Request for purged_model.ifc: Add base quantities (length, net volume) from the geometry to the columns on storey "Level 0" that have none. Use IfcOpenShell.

First a look at what the model holds.

```python
import ifcopenshell
import ifcopenshell.util.element
import ifcopenshell.util.unit

model = ifcopenshell.open("purged_model.ifc")
print(model.schema)
for unit_type in ("LENGTHUNIT", "AREAUNIT", "VOLUMEUNIT"):
    print(unit_type, ifcopenshell.util.unit.calculate_unit_scale(model, unit_type))
storey = next(s for s in model.by_type("IfcBuildingStorey") if s.Name == "Level 0")
columns = [e for e in ifcopenshell.util.element.get_decomposition(storey) if e.is_a("IfcColumn")]
for e in sorted(columns, key=lambda e: e.id()):
    print(e.id(), e.is_a(), e.Name, list(ifcopenshell.util.element.get_psets(e, qtos_only=True)), sep=" | ")
```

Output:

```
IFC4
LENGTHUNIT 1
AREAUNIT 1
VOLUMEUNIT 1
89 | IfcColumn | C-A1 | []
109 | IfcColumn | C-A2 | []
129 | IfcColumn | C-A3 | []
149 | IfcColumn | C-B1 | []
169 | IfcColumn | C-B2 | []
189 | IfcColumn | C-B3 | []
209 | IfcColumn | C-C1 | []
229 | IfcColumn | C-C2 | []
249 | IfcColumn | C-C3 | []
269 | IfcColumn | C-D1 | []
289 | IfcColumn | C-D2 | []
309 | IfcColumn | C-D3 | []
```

```python
import ifcopenshell
import ifcopenshell.api.pset
import ifcopenshell.geom
import ifcopenshell.util.element
import ifcopenshell.util.shape
import ifcopenshell.util.unit

model = ifcopenshell.open("purged_model.ifc")
unit_scale = ifcopenshell.util.unit.calculate_unit_scale(model)
volume_scale = ifcopenshell.util.unit.calculate_unit_scale(model, "VOLUMEUNIT")
settings = ifcopenshell.geom.settings()

storey = next(s for s in model.by_type("IfcBuildingStorey") if s.Name == "Level 0")
columns = [e for e in ifcopenshell.util.element.get_decomposition(storey) if e.is_a("IfcColumn")]

for e in sorted(columns, key=lambda e: e.id()):
    if ifcopenshell.util.element.get_psets(e, qtos_only=True, should_inherit=False):
        continue
    # Geometry comes back in metres, in the element's own axes.
    shape = ifcopenshell.geom.create_shape(settings, e)
    values = {
        "Length": ifcopenshell.util.shape.get_z(shape.geometry) / unit_scale,
        "NetVolume": ifcopenshell.util.shape.get_volume(shape.geometry) / volume_scale,
    }
    qto = ifcopenshell.api.pset.add_qto(model, product=e, name="Qto_ColumnBaseQuantities")
    ifcopenshell.api.pset.edit_qto(model, qto=qto, properties=values)
    print(e.id(), {k: round(v, 3) for k, v in values.items()})

model.write("purged_model_edited.ifc")
```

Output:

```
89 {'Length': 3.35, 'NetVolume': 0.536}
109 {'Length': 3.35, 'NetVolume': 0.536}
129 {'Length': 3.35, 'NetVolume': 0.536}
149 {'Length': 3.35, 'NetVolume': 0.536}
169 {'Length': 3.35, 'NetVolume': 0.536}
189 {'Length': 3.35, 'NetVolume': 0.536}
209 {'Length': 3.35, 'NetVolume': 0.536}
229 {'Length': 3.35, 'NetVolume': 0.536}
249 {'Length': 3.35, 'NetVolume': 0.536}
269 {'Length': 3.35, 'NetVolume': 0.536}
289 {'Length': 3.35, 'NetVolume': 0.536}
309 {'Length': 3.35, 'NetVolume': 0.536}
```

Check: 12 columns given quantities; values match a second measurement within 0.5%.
